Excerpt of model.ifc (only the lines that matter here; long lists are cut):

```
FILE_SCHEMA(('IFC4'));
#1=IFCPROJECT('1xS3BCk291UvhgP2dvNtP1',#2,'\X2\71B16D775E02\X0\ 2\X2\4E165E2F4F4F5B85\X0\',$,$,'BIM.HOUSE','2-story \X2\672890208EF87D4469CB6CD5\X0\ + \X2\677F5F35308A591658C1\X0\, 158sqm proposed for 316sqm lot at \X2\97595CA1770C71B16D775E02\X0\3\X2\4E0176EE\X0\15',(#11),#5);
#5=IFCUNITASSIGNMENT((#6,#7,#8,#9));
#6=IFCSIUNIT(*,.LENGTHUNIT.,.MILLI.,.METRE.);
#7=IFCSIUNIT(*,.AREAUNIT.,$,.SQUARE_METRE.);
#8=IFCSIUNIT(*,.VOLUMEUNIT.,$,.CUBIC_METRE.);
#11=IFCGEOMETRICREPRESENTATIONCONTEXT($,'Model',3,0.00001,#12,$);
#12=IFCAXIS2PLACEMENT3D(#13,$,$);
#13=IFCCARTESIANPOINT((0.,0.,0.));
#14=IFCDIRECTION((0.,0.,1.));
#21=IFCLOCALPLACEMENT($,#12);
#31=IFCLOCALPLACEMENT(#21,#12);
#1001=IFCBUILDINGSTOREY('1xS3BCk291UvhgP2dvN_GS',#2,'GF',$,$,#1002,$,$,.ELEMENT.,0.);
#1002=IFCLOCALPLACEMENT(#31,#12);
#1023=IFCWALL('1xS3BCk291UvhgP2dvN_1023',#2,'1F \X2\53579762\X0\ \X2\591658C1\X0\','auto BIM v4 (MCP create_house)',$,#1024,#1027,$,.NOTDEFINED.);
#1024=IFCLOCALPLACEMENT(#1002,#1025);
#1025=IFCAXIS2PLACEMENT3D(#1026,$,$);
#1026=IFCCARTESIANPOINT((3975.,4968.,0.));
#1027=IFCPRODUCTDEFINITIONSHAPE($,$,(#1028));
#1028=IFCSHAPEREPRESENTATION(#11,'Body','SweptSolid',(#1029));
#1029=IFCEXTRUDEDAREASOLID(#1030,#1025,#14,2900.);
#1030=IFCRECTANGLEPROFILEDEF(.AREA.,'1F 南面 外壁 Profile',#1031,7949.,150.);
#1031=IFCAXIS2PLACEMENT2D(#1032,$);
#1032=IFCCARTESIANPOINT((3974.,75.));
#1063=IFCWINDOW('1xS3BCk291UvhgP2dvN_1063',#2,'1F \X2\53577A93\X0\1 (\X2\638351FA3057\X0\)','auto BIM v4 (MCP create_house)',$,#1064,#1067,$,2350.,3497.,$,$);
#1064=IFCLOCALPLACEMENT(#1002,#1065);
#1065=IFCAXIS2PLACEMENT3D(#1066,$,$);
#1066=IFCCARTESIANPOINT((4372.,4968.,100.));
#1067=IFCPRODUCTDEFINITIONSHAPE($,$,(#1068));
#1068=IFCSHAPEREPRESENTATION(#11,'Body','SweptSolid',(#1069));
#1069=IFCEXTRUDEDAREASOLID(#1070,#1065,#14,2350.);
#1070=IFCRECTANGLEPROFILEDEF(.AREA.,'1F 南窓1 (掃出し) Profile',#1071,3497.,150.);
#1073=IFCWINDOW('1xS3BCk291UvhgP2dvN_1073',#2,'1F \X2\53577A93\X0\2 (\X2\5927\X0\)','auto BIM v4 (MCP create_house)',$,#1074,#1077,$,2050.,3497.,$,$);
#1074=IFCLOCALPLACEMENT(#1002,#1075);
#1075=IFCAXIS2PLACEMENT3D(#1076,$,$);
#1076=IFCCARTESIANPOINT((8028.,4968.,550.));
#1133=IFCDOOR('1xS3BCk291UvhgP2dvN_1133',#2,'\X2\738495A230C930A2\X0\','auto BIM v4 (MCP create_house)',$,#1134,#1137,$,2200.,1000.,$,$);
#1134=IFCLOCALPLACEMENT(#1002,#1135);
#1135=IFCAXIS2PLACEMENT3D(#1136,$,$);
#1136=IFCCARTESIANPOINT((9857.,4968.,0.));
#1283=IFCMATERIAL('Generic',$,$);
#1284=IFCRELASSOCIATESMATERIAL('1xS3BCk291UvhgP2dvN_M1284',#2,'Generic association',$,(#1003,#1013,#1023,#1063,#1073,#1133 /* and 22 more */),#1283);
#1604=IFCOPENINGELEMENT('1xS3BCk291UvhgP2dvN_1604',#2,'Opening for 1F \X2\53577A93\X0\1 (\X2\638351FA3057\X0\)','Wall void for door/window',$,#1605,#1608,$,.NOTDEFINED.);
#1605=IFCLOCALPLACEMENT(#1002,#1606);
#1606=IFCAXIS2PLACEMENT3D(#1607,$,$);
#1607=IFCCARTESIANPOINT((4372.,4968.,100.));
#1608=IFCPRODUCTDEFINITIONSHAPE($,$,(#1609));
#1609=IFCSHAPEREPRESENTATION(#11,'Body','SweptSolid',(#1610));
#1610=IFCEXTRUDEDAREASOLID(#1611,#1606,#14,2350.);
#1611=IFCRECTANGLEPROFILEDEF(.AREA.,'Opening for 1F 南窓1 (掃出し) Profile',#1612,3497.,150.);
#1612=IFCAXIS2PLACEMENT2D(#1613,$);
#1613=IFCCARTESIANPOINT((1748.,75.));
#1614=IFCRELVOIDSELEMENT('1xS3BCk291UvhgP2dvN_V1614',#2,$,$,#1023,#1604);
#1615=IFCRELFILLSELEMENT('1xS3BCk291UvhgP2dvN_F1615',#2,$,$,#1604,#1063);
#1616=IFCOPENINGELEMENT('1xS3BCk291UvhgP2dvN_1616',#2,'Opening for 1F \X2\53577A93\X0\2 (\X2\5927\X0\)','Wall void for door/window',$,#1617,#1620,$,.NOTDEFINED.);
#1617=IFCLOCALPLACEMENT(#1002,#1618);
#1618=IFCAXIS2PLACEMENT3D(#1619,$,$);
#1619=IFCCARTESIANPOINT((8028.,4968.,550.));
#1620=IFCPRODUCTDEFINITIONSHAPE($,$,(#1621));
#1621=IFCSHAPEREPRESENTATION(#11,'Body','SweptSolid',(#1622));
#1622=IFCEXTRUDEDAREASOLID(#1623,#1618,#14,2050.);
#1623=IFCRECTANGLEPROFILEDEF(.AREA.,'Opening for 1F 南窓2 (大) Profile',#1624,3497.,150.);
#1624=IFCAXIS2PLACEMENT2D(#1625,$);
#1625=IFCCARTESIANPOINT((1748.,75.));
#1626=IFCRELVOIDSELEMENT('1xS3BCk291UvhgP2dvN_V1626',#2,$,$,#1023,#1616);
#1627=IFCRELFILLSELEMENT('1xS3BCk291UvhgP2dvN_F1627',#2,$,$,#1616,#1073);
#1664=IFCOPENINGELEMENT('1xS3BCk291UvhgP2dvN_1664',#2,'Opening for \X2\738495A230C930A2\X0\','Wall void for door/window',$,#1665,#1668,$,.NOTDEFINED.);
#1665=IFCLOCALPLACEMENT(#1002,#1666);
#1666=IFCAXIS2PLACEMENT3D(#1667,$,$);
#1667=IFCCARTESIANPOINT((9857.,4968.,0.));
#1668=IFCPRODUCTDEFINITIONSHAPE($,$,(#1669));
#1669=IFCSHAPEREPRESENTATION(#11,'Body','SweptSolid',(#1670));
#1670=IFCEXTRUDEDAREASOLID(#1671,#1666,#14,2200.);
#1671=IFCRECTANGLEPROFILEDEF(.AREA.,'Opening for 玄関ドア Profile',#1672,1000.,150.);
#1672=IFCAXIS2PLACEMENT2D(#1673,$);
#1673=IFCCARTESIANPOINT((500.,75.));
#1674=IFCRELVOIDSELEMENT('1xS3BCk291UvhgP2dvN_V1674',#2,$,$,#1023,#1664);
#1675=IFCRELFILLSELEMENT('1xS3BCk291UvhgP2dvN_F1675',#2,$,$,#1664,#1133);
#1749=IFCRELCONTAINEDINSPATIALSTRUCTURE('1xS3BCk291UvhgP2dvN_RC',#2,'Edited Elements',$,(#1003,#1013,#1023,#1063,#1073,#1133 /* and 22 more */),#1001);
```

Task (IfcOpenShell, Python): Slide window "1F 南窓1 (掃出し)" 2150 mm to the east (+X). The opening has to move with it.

```python
import ifcopenshell
import ifcopenshell.api.geometry
import ifcopenshell.util.placement

model = ifcopenshell.open("model.ifc")

window = model.by_id(1063)
opening = window.FillsVoids[0].RelatingOpeningElement
wall = opening.VoidsElements[0].RelatingBuildingElement

wall_matrix = ifcopenshell.util.placement.get_local_placement(wall.ObjectPlacement)
shift = wall_matrix[:3, 0] * 2150.0
before = ifcopenshell.util.placement.get_local_placement(window.ObjectPlacement)[:3, 3].copy()

# The window is not placed relative to its opening, so move both.
for product in (opening, window):
    matrix = ifcopenshell.util.placement.get_local_placement(product.ObjectPlacement)
    matrix[:3, 3] += shift
    ifcopenshell.api.geometry.edit_object_placement(model, product=product, matrix=matrix, is_si=False)

after = ifcopenshell.util.placement.get_local_placement(window.ObjectPlacement)[:3, 3]
print("window moved by", (after - before).round(3) + 0.0)

model.write("model-out.ifc")
```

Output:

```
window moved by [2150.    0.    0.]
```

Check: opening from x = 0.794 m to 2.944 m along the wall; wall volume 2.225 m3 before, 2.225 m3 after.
